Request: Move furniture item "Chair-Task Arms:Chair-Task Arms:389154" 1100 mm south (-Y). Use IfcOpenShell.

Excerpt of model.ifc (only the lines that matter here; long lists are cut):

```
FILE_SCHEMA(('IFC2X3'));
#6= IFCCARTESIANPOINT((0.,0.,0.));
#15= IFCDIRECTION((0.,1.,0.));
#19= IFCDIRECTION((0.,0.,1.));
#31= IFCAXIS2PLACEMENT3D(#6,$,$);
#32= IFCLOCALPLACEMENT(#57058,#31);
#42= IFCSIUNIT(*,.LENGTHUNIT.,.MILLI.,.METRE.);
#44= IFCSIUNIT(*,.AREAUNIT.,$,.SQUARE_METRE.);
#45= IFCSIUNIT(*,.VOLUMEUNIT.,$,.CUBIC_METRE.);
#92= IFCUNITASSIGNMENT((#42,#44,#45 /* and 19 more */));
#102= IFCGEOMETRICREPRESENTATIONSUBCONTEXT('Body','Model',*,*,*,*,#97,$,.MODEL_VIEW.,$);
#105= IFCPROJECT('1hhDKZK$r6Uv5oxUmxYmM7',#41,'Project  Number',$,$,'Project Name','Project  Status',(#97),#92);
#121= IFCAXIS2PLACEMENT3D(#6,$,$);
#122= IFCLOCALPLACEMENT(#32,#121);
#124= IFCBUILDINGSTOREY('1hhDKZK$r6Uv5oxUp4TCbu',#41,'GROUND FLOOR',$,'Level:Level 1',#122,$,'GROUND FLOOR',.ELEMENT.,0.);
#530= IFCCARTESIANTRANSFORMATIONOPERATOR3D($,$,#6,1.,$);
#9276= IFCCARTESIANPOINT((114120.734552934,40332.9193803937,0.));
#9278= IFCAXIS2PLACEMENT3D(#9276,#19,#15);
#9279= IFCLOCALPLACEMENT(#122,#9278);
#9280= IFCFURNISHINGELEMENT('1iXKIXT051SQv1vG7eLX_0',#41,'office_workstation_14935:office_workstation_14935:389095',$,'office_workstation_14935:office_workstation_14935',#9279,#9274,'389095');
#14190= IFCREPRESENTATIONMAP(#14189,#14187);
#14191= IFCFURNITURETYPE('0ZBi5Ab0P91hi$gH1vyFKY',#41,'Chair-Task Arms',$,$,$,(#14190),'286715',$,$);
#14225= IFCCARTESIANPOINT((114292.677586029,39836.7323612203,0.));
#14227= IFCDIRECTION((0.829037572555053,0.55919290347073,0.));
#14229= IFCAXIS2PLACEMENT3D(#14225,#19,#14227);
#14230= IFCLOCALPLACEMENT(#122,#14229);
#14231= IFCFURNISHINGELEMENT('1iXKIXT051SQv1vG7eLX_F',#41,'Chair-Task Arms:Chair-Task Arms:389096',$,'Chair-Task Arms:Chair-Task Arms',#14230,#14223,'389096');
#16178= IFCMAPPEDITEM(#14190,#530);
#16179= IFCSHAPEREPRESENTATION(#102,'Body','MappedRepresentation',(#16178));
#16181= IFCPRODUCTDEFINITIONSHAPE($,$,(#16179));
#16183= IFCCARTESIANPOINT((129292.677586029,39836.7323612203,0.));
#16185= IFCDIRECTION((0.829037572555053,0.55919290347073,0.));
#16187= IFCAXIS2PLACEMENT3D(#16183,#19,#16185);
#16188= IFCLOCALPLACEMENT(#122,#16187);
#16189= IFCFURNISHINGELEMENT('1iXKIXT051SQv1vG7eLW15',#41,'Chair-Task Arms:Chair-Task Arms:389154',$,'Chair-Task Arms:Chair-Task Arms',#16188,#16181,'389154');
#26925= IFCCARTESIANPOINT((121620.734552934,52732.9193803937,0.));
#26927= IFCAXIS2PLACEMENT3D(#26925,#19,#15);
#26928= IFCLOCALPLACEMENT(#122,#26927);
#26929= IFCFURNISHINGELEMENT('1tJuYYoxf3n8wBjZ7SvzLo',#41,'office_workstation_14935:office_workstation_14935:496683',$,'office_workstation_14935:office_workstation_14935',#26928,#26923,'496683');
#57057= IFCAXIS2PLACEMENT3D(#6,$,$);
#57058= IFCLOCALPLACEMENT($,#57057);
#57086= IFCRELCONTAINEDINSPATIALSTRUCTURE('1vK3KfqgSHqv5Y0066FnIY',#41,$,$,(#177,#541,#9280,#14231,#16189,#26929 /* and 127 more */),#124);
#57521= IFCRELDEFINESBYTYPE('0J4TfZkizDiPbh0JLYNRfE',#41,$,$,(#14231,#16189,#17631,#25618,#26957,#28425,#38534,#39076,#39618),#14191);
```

```python
import ifcopenshell
import ifcopenshell.api.geometry
import ifcopenshell.util.placement

model = ifcopenshell.open("model.ifc")

item = model.by_guid("1iXKIXT051SQv1vG7eLW15")
matrix = ifcopenshell.util.placement.get_local_placement(item.ObjectPlacement)
matrix[1, 3] -= 1100.0
ifcopenshell.api.geometry.edit_object_placement(model, product=item, matrix=matrix, is_si=False)

print(ifcopenshell.util.placement.get_local_placement(item.ObjectPlacement).round(3) + 0.0)

model.write("model_edited.ifc")
```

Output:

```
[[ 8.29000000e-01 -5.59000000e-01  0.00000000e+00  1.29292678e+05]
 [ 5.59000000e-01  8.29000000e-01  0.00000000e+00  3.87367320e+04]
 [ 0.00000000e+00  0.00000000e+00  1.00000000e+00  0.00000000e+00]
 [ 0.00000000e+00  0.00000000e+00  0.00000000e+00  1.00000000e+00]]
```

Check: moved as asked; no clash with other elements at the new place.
